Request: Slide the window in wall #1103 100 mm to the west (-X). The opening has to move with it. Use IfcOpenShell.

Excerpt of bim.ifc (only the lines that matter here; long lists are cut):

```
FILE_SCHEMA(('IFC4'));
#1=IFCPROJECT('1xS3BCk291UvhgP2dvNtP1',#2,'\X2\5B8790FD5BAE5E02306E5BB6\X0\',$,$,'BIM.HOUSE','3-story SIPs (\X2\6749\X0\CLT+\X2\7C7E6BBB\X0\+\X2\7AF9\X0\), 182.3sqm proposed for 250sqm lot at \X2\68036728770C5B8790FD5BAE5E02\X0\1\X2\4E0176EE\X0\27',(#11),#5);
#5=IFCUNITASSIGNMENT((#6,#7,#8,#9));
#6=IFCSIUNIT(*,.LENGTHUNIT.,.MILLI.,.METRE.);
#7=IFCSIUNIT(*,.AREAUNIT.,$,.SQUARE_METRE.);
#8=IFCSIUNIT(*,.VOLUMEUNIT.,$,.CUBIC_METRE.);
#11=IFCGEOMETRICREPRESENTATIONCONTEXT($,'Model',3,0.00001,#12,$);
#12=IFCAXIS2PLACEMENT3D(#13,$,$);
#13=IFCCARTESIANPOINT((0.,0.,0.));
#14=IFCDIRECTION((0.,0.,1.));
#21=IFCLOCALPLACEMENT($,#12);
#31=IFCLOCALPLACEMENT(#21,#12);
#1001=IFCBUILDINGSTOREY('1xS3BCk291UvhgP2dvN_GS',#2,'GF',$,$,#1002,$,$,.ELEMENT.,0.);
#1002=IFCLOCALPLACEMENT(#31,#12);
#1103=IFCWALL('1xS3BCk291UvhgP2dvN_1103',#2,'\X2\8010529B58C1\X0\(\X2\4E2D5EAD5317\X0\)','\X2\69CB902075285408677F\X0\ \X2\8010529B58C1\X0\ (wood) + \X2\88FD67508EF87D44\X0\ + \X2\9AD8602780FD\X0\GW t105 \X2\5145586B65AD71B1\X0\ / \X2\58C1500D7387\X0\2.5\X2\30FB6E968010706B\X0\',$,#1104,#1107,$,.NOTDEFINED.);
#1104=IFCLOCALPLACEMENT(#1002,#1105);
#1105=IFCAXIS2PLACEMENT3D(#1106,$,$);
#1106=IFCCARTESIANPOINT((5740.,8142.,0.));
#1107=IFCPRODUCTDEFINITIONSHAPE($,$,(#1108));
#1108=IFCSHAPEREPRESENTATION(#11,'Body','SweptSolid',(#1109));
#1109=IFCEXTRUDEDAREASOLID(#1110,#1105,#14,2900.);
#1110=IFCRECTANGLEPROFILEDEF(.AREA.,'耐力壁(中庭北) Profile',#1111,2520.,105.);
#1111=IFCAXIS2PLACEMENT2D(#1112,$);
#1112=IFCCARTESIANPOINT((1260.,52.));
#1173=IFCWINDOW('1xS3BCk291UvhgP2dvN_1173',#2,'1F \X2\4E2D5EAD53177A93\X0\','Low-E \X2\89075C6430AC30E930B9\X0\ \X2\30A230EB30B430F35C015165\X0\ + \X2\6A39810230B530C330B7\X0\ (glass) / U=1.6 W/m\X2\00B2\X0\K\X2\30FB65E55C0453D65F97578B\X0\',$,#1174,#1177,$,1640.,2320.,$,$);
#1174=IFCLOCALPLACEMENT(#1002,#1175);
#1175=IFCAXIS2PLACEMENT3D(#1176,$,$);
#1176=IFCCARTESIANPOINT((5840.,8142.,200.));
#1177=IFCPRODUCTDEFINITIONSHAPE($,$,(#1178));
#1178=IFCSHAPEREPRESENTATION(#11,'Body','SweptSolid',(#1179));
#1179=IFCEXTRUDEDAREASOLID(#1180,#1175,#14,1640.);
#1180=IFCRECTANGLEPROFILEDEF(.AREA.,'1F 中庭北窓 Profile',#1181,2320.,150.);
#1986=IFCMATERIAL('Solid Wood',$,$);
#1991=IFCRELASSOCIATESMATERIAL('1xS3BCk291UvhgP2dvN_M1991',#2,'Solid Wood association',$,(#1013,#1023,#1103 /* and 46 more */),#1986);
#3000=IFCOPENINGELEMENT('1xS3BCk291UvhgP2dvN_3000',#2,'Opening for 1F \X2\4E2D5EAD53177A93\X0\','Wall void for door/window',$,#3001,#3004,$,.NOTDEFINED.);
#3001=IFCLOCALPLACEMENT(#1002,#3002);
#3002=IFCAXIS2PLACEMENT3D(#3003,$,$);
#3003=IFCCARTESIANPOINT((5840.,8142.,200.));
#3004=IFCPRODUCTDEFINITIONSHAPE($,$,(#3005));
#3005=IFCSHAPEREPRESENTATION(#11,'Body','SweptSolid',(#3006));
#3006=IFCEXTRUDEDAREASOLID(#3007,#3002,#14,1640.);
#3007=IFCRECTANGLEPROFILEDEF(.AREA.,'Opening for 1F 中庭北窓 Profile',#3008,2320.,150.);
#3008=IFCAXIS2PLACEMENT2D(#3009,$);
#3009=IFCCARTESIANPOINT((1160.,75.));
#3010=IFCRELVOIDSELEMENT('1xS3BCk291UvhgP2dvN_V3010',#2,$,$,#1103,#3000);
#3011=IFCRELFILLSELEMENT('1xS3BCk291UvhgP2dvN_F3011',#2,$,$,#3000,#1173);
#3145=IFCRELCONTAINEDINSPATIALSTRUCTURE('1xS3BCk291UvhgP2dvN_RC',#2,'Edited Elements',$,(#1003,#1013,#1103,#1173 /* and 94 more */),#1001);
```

```python
import ifcopenshell
import ifcopenshell.api.geometry
import ifcopenshell.util.placement

model = ifcopenshell.open("bim.ifc")

window = model.by_guid("1xS3BCk291UvhgP2dvN_1173")
opening = window.FillsVoids[0].RelatingOpeningElement
wall = opening.VoidsElements[0].RelatingBuildingElement

wall_matrix = ifcopenshell.util.placement.get_local_placement(wall.ObjectPlacement)
shift = wall_matrix[:3, 0] * -100.0
before = ifcopenshell.util.placement.get_local_placement(window.ObjectPlacement)[:3, 3].copy()

# The window is not placed relative to its opening, so move both.
for product in (opening, window):
    matrix = ifcopenshell.util.placement.get_local_placement(product.ObjectPlacement)
    matrix[:3, 3] += shift
    ifcopenshell.api.geometry.edit_object_placement(model, product=product, matrix=matrix, is_si=False)

after = ifcopenshell.util.placement.get_local_placement(window.ObjectPlacement)[:3, 3]
print("window moved by", (after - before).round(3) + 0.0)

model.write("bim_v2.ifc")
```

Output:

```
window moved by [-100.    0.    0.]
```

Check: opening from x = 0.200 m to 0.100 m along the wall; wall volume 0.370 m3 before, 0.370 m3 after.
